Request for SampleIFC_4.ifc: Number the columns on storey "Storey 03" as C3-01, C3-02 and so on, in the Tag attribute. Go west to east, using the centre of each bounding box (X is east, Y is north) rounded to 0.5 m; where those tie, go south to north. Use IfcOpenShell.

First a look at what the model holds.

```python
import ifcopenshell
import ifcopenshell.util.element
import ifcopenshell.util.placement

model = ifcopenshell.open("SampleIFC_4.ifc")
print(model.schema)
storey = next(s for s in model.by_type("IfcBuildingStorey") if s.Name == "Storey 03")
columns = [e for e in ifcopenshell.util.element.get_decomposition(storey) if e.is_a("IfcColumn")]
for e in sorted(columns, key=lambda e: e.id()):
    origin = ifcopenshell.util.placement.get_local_placement(e.ObjectPlacement)[:3, 3]
    print(e.id(), e.Tag, e.Name, origin.round(2) + 0.0, sep=" | ")
```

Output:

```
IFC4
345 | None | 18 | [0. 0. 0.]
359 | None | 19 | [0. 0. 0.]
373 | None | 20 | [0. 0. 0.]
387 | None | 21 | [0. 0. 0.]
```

```python
import ifcopenshell
import ifcopenshell.geom
import ifcopenshell.util.element
import ifcopenshell.util.shape

model = ifcopenshell.open("SampleIFC_4.ifc")
settings = ifcopenshell.geom.settings()
settings.set("use-world-coords", True)


def centre(element):
    shape = ifcopenshell.geom.create_shape(settings, element)
    return ifcopenshell.util.shape.get_bbox_centroid(shape.geometry)


storey = next(s for s in model.by_type("IfcBuildingStorey") if s.Name == "Storey 03")
columns = [e for e in ifcopenshell.util.element.get_decomposition(storey) if e.is_a("IfcColumn")]

# Insertion points can sit at a corner or the storey origin, so sort by the geometry (in metres).
centres = {e: centre(e) for e in columns}
columns.sort(key=lambda e: (round(centres[e][0] / 0.5), centres[e][1]))

for i, e in enumerate(columns, start=1):
    number = f"C3-{i:02d}"
    e.Tag = number
    print(e.id(), number)

model.write("SampleIFC_4-out.ifc")
```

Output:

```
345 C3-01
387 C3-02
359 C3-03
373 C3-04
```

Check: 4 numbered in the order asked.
